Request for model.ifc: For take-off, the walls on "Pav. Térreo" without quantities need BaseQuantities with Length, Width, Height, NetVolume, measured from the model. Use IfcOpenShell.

First a look at what the model holds.

```python
import ifcopenshell
import ifcopenshell.util.element
import ifcopenshell.util.unit

model = ifcopenshell.open("model.ifc")
print(model.schema)
for unit_type in ("LENGTHUNIT", "AREAUNIT", "VOLUMEUNIT"):
    print(unit_type, ifcopenshell.util.unit.calculate_unit_scale(model, unit_type))
storey = next(s for s in model.by_type("IfcBuildingStorey") if s.Name == "Pav. Térreo")
walls = [e for e in ifcopenshell.util.element.get_decomposition(storey) if e.is_a("IfcWall")]
for e in sorted(walls, key=lambda e: e.id()):
    print(e.id(), e.is_a(), e.Name, list(ifcopenshell.util.element.get_psets(e, qtos_only=True)), sep=" | ")
```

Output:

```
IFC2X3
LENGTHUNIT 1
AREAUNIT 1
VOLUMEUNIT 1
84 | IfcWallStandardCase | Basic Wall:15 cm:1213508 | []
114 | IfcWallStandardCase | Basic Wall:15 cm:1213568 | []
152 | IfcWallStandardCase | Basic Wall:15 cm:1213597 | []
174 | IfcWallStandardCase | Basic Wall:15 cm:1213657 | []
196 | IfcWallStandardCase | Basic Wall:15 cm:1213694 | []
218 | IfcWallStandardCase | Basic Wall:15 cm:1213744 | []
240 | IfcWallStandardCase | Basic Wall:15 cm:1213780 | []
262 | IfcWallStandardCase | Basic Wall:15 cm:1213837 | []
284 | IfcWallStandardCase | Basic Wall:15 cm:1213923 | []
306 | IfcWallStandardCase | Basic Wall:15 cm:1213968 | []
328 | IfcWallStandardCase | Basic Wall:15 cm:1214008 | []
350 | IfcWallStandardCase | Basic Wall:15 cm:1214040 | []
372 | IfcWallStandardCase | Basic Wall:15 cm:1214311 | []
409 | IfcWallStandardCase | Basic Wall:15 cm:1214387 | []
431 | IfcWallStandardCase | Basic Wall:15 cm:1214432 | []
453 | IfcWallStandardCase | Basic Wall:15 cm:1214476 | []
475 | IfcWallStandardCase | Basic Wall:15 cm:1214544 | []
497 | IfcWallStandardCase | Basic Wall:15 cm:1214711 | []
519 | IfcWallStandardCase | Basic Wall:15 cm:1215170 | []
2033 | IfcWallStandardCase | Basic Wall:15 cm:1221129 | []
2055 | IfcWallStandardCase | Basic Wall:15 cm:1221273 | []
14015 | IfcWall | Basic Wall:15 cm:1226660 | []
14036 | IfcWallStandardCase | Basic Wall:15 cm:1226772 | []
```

```python
import ifcopenshell
import ifcopenshell.api.pset
import ifcopenshell.geom
import ifcopenshell.util.element
import ifcopenshell.util.shape
import ifcopenshell.util.unit

model = ifcopenshell.open("model.ifc")
unit_scale = ifcopenshell.util.unit.calculate_unit_scale(model)
volume_scale = ifcopenshell.util.unit.calculate_unit_scale(model, "VOLUMEUNIT")
settings = ifcopenshell.geom.settings()

storey = next(s for s in model.by_type("IfcBuildingStorey") if s.Name == "Pav. Térreo")
walls = [e for e in ifcopenshell.util.element.get_decomposition(storey) if e.is_a("IfcWall")]

for e in sorted(walls, key=lambda e: e.id()):
    if ifcopenshell.util.element.get_psets(e, qtos_only=True, should_inherit=False):
        continue
    # Geometry comes back in metres, in the element's own axes.
    shape = ifcopenshell.geom.create_shape(settings, e)
    values = {
        "Length": ifcopenshell.util.shape.get_x(shape.geometry) / unit_scale,
        "Width": ifcopenshell.util.shape.get_y(shape.geometry) / unit_scale,
        "Height": ifcopenshell.util.shape.get_z(shape.geometry) / unit_scale,
        "NetVolume": ifcopenshell.util.shape.get_volume(shape.geometry) / volume_scale,
    }
    qto = ifcopenshell.api.pset.add_qto(model, product=e, name="BaseQuantities")
    ifcopenshell.api.pset.edit_qto(model, qto=qto, properties=values)
    print(e.id(), {k: round(v, 3) for k, v in values.items()})

model.write("model_rev.ifc")
```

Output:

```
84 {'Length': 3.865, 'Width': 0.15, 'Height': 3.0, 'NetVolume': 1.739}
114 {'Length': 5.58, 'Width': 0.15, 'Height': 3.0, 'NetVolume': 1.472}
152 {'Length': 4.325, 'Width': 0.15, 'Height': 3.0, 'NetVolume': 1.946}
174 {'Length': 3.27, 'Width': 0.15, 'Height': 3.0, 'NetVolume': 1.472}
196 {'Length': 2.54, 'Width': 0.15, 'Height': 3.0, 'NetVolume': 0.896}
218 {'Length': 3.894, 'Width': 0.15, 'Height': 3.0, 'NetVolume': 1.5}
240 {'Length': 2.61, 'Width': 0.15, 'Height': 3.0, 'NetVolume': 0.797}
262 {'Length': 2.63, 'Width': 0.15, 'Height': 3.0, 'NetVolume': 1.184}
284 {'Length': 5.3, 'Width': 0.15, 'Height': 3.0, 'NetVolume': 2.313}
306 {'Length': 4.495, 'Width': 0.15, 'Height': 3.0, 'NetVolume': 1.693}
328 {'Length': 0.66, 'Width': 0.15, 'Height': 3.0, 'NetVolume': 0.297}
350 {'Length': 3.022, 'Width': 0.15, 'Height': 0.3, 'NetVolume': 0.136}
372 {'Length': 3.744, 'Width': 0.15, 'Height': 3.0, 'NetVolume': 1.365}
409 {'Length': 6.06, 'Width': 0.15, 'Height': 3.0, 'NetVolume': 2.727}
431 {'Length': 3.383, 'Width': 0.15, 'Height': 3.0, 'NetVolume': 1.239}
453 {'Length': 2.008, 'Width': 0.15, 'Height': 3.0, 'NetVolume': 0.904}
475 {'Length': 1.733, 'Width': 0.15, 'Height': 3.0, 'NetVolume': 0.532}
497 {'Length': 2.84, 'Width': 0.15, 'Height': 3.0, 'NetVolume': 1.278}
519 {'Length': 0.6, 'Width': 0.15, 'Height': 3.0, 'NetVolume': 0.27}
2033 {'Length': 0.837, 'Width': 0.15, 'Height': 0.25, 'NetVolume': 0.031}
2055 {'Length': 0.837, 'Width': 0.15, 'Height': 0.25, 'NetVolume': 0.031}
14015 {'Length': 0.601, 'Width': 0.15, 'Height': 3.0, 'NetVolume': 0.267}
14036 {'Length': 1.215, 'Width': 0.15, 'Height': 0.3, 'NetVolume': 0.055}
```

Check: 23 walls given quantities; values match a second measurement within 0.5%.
